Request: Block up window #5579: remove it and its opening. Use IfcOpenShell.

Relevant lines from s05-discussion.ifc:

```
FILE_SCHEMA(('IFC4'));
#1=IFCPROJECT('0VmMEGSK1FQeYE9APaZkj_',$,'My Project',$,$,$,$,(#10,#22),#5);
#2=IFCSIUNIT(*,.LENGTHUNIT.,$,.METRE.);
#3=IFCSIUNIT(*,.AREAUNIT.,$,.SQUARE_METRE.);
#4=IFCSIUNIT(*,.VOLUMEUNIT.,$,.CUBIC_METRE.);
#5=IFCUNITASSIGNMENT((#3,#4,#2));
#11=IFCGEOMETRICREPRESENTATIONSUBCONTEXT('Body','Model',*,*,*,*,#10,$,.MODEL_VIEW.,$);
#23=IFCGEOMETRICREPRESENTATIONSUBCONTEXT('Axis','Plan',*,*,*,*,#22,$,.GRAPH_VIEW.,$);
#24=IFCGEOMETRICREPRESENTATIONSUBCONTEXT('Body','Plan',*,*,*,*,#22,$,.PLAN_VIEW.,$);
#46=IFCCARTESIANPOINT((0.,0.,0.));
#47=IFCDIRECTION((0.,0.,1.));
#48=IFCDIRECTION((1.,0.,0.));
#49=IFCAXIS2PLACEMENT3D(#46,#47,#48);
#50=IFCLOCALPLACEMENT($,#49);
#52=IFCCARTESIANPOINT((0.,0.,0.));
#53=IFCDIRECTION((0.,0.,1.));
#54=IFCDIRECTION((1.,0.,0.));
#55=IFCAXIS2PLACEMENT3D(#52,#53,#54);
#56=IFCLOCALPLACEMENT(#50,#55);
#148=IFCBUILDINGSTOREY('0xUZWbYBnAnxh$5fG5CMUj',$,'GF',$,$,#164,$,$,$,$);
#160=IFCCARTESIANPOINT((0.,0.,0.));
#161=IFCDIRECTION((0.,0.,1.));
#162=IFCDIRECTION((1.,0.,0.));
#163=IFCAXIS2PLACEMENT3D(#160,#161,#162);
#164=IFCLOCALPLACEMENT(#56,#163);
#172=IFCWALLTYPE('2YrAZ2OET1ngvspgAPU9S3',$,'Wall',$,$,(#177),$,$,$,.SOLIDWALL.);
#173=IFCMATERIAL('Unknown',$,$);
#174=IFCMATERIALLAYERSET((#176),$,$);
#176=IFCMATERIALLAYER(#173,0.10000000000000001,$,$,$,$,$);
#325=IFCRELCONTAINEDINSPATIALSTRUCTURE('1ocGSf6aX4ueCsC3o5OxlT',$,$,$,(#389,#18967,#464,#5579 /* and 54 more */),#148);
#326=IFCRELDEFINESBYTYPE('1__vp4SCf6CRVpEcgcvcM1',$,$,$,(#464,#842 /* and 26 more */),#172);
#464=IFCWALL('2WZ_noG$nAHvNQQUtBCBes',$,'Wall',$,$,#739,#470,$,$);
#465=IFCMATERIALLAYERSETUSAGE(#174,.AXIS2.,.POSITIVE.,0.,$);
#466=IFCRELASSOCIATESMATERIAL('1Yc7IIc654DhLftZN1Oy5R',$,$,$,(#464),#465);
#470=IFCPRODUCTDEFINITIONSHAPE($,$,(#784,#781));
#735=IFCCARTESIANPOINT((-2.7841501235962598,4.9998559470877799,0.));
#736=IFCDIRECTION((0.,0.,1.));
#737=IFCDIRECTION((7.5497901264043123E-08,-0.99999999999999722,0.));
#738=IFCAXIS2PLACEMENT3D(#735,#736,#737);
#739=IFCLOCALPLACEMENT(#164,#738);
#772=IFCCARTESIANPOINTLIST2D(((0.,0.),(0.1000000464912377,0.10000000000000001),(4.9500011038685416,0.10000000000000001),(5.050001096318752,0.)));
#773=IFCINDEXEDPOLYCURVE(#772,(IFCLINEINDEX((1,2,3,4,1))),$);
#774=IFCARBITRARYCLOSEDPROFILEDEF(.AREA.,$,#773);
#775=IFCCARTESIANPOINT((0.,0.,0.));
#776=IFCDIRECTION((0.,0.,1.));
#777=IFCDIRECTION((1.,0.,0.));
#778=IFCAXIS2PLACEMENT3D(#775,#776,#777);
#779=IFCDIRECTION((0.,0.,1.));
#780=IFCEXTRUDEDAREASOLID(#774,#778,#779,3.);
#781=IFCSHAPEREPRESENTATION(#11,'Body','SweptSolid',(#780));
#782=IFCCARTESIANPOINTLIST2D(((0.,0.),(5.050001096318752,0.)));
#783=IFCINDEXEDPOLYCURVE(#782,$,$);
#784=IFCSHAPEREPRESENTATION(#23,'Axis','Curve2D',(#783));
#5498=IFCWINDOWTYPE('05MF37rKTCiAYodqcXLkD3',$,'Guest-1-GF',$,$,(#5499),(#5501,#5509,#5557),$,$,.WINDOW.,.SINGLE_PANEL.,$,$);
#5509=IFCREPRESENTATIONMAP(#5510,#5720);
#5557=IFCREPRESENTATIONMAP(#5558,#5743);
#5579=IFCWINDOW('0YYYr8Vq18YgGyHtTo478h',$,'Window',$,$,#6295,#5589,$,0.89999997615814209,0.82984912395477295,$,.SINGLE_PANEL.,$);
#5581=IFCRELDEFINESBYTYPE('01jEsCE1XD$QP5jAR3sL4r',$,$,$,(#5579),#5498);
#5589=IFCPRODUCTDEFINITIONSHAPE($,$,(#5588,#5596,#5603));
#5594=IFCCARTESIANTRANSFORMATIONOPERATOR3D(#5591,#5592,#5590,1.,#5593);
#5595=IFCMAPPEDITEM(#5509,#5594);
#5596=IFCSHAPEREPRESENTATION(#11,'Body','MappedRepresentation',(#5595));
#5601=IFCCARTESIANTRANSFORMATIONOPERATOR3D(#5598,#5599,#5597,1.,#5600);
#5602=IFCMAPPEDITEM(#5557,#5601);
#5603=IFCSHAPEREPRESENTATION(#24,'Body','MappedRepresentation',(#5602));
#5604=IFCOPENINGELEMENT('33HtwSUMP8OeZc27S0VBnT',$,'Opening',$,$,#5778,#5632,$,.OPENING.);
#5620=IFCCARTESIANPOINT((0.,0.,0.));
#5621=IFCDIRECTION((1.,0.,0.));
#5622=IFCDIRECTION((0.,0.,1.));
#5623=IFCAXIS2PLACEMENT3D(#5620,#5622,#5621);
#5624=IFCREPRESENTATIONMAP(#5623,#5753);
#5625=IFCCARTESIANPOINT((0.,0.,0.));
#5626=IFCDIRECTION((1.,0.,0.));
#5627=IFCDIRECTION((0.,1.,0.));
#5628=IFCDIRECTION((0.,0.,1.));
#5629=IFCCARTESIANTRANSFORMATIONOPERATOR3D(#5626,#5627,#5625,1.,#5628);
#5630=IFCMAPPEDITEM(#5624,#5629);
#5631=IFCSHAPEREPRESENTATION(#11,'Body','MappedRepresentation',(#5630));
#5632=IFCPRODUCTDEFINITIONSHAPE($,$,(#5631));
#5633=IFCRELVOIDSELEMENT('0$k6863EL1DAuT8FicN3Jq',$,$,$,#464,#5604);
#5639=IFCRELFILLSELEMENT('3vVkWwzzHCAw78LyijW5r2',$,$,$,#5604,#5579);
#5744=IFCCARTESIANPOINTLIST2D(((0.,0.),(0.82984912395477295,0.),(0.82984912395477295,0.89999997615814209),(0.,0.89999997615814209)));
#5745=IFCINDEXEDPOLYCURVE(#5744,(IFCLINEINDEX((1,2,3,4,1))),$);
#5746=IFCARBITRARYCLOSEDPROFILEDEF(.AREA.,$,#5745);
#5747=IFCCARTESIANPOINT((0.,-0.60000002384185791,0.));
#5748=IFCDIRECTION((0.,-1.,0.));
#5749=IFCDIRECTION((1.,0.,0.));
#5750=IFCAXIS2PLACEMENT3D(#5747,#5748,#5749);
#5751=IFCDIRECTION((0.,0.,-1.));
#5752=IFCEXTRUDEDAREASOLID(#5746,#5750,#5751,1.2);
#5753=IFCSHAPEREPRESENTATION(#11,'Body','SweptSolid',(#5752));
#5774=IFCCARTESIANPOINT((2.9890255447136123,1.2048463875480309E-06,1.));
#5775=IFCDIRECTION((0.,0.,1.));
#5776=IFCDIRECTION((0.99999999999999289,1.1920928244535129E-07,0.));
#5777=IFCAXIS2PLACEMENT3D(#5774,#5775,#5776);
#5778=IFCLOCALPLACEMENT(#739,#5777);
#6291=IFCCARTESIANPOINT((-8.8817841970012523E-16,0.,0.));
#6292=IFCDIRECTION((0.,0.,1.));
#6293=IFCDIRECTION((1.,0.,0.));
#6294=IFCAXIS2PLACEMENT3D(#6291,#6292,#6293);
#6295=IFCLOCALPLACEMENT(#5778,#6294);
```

```python
import ifcopenshell
import ifcopenshell.api.feature
import ifcopenshell.api.root
import ifcopenshell.geom
import ifcopenshell.util.shape

model = ifcopenshell.open("s05-discussion.ifc")
settings = ifcopenshell.geom.settings()


def volume(element):
    """Net volume in cubic metres, openings subtracted."""
    shape = ifcopenshell.geom.create_shape(settings, element)
    return ifcopenshell.util.shape.get_volume(shape.geometry)


window = model.by_id(5579)
opening = window.FillsVoids[0].RelatingOpeningElement
wall = opening.VoidsElements[0].RelatingBuildingElement
before = volume(wall)

ifcopenshell.api.root.remove_product(model, product=window)
ifcopenshell.api.feature.remove_feature(model, feature=opening)

after = volume(wall)

print(f"wall volume {before:.3f} -> {after:.3f} m3")

model.write("s05-discussion-out.ifc")
```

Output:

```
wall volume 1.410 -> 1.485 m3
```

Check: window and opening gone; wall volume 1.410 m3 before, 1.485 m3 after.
